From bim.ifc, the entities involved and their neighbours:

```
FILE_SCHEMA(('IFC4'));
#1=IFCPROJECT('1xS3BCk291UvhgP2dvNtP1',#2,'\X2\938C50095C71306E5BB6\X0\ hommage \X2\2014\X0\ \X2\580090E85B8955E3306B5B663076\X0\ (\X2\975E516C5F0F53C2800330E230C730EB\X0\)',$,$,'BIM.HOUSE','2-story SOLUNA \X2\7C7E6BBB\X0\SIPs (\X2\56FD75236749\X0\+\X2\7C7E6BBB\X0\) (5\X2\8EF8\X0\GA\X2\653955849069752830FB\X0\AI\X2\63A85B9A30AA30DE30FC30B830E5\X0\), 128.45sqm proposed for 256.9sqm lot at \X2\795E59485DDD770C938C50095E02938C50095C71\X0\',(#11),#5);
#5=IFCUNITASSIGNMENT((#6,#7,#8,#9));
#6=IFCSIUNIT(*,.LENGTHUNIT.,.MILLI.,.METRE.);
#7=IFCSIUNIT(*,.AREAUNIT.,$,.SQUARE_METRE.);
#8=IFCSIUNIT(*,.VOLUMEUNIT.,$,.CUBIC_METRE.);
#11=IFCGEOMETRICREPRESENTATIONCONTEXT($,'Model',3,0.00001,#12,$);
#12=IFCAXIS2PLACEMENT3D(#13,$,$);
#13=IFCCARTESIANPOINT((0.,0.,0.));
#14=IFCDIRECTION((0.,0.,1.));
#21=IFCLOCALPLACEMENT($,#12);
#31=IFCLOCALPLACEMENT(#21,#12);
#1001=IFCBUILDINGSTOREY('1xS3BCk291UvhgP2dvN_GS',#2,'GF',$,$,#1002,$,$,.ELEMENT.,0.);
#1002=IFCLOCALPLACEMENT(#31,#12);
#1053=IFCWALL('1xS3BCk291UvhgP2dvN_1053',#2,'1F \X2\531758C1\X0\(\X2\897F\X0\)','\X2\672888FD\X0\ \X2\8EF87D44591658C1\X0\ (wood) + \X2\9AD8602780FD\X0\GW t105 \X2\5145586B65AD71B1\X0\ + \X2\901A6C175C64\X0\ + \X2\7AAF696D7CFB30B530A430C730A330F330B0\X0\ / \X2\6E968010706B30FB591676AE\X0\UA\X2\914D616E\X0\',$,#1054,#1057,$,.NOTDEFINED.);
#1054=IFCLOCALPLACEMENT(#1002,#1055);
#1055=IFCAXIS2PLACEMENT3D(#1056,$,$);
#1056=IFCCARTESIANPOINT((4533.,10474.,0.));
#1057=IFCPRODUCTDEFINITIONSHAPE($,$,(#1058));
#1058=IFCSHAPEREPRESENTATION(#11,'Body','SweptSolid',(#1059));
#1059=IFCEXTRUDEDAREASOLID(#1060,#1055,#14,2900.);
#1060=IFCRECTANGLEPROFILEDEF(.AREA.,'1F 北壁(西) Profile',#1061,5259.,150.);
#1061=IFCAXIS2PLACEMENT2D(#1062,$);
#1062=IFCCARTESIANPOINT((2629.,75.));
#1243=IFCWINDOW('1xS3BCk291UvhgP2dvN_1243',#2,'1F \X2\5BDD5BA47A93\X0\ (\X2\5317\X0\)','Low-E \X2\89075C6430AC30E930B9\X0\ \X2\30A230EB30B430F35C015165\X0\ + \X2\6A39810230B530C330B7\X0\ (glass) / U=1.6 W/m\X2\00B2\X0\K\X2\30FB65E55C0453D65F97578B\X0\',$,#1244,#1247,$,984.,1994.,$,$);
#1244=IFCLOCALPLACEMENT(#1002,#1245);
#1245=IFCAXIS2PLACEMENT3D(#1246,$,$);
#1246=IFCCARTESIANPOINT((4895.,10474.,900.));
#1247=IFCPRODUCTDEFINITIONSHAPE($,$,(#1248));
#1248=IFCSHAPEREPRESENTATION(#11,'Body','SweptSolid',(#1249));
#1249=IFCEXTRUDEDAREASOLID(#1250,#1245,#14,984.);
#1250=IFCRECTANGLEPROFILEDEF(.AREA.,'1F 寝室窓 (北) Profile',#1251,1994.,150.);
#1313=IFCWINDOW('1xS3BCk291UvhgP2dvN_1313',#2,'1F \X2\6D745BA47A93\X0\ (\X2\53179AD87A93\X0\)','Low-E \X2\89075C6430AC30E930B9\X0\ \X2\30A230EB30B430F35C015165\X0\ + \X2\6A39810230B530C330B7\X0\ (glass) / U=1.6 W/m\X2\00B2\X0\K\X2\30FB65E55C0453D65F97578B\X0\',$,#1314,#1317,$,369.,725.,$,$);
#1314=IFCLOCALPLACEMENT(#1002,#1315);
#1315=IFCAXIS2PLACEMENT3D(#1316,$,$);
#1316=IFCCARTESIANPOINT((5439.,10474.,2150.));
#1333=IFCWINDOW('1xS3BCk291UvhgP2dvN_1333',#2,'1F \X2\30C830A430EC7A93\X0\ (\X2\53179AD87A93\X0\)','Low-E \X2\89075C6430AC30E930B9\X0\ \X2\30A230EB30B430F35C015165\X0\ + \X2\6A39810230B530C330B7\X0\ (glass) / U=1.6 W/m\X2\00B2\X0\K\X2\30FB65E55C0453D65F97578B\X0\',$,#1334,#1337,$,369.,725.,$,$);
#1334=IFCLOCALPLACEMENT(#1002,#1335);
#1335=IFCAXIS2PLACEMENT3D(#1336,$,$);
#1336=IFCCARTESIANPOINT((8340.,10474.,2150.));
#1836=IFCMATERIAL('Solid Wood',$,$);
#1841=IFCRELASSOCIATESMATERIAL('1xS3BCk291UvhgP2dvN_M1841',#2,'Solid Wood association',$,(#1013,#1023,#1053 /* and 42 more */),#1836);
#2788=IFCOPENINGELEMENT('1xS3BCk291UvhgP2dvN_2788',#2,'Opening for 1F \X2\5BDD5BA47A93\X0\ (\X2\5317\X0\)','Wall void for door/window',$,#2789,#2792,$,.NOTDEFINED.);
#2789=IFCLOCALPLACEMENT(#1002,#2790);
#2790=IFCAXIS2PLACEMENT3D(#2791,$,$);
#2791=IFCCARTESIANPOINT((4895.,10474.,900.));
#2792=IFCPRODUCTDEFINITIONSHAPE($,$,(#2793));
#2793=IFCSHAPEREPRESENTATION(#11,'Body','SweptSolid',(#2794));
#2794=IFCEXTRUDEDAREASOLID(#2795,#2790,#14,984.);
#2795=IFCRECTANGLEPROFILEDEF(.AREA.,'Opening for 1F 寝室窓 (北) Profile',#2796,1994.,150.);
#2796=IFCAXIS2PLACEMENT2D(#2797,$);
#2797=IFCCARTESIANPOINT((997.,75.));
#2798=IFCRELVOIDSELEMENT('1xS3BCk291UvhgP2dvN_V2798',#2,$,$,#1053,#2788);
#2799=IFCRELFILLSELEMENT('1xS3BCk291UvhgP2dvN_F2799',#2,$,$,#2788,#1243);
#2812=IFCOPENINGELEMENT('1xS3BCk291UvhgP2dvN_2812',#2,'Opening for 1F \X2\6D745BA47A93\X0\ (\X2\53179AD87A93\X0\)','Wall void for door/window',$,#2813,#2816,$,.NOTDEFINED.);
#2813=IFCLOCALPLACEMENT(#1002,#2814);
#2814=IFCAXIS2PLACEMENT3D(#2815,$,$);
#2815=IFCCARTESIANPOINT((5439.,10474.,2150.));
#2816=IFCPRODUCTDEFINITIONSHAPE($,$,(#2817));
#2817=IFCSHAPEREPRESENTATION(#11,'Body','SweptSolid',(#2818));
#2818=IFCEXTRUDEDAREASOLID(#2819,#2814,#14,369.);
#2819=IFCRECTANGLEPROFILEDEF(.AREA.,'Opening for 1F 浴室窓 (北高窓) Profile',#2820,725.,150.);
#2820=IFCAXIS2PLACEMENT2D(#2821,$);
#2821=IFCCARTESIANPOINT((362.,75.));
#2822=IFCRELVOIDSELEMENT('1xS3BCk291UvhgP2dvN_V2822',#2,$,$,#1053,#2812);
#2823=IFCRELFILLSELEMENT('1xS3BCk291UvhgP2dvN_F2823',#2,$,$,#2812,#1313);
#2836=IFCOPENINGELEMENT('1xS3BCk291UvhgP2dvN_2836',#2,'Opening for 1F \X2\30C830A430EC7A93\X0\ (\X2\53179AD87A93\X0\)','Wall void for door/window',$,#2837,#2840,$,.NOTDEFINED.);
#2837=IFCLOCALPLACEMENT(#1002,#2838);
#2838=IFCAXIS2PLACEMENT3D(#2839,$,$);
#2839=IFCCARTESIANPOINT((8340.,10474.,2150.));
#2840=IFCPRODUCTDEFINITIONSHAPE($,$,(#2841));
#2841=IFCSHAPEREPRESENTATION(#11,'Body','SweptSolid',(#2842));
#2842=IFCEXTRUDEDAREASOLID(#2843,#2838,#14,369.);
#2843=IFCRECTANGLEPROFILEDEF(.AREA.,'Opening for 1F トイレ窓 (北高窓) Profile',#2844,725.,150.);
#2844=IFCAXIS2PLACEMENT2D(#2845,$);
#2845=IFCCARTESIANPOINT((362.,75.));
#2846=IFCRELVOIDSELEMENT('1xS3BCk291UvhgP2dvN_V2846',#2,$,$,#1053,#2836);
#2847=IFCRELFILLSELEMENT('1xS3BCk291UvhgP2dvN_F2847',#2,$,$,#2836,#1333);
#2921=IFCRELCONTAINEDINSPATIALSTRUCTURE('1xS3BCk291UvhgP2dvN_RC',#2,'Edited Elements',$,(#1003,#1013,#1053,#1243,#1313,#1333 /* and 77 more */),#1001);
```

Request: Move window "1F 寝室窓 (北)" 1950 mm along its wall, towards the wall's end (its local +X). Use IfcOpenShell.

```python
import ifcopenshell
import ifcopenshell.api.geometry
import ifcopenshell.util.placement
import ifcopenshell.util.unit

model = ifcopenshell.open("bim.ifc")
unit_scale = ifcopenshell.util.unit.calculate_unit_scale(model)

window = model.by_guid("1xS3BCk291UvhgP2dvN_1243")
opening = window.FillsVoids[0].RelatingOpeningElement
wall = opening.VoidsElements[0].RelatingBuildingElement

wall_matrix = ifcopenshell.util.placement.get_local_placement(wall.ObjectPlacement)
shift = wall_matrix[:3, 0] * 1.95 / unit_scale
before = ifcopenshell.util.placement.get_local_placement(window.ObjectPlacement)[:3, 3].copy()

# The window is not placed relative to its opening, so move both.
for product in (opening, window):
    matrix = ifcopenshell.util.placement.get_local_placement(product.ObjectPlacement)
    matrix[:3, 3] += shift
    ifcopenshell.api.geometry.edit_object_placement(model, product=product, matrix=matrix, is_si=False)

after = ifcopenshell.util.placement.get_local_placement(window.ObjectPlacement)[:3, 3]
print("window moved by", (after - before).round(3) + 0.0)

model.write("bim_edited.ifc")
```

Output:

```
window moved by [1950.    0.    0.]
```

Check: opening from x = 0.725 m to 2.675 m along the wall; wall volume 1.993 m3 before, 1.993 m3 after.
